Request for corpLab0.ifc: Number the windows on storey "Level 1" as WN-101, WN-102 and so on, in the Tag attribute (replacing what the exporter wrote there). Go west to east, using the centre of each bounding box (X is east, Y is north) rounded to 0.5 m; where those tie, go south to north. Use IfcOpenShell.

First a look at what the model holds.

```python
import ifcopenshell
import ifcopenshell.util.element
import ifcopenshell.util.placement

model = ifcopenshell.open("corpLab0.ifc")
print(model.schema)
storey = next(s for s in model.by_type("IfcBuildingStorey") if s.Name == "Level 1")
windows = [e for e in ifcopenshell.util.element.get_decomposition(storey) if e.is_a("IfcWindow")]
for e in sorted(windows, key=lambda e: e.id()):
    origin = ifcopenshell.util.placement.get_local_placement(e.ObjectPlacement)[:3, 3]
    print(e.id(), e.Tag, e.Name, origin.round(2) + 0.0, sep=" | ")
```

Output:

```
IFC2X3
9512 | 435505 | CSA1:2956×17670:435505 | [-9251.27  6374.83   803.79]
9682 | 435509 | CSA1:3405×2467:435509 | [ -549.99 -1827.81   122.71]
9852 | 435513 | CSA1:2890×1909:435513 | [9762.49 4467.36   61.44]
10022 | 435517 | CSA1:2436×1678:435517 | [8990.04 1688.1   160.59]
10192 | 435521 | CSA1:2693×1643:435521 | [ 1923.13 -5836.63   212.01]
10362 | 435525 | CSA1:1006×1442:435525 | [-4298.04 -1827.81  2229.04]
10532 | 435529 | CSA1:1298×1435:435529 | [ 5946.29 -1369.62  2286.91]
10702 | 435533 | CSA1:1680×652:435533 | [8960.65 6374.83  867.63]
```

```python
import ifcopenshell
import ifcopenshell.geom
import ifcopenshell.util.element
import ifcopenshell.util.shape

model = ifcopenshell.open("corpLab0.ifc")
settings = ifcopenshell.geom.settings()
settings.set("use-world-coords", True)


def centre(element):
    shape = ifcopenshell.geom.create_shape(settings, element)
    return ifcopenshell.util.shape.get_bbox_centroid(shape.geometry)


storey = next(s for s in model.by_type("IfcBuildingStorey") if s.Name == "Level 1")
windows = [e for e in ifcopenshell.util.element.get_decomposition(storey) if e.is_a("IfcWindow")]

# Insertion points can sit at a corner or the storey origin, so sort by the geometry (in metres).
centres = {e: centre(e) for e in windows}
windows.sort(key=lambda e: (round(centres[e][0] / 0.5), centres[e][1]))

for i, e in enumerate(windows, start=1):
    number = f"WN-1{i:02d}"
    e.Tag = number
    print(e.id(), number)

model.write("corpLab0_edited.ifc")
```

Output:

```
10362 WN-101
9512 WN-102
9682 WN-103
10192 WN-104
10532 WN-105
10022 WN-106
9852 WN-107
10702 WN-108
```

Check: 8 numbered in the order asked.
